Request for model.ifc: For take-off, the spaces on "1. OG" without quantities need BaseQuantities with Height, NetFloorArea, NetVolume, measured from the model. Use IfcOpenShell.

First a look at what the model holds.

```python
import ifcopenshell
import ifcopenshell.util.element
import ifcopenshell.util.unit

model = ifcopenshell.open("model.ifc")
print(model.schema)
for unit_type in ("LENGTHUNIT", "AREAUNIT", "VOLUMEUNIT"):
    print(unit_type, ifcopenshell.util.unit.calculate_unit_scale(model, unit_type))
storey = next(s for s in model.by_type("IfcBuildingStorey") if s.Name == "1. OG")
spaces = [e for e in ifcopenshell.util.element.get_decomposition(storey) if e.is_a("IfcSpace")]
for e in sorted(spaces, key=lambda e: e.id()):
    print(e.id(), e.is_a(), e.Name, list(ifcopenshell.util.element.get_psets(e, qtos_only=True)), sep=" | ")
```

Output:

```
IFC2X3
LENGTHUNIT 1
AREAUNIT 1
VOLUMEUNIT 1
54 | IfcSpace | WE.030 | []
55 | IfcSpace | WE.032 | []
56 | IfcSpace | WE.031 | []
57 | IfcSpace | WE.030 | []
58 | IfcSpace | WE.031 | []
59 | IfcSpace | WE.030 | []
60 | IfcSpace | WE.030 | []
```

```python
import ifcopenshell
import ifcopenshell.api.pset
import ifcopenshell.geom
import ifcopenshell.util.element
import ifcopenshell.util.shape
import ifcopenshell.util.unit

model = ifcopenshell.open("model.ifc")
unit_scale = ifcopenshell.util.unit.calculate_unit_scale(model)
area_scale = ifcopenshell.util.unit.calculate_unit_scale(model, "AREAUNIT")
volume_scale = ifcopenshell.util.unit.calculate_unit_scale(model, "VOLUMEUNIT")
settings = ifcopenshell.geom.settings()

storey = next(s for s in model.by_type("IfcBuildingStorey") if s.Name == "1. OG")
spaces = [e for e in ifcopenshell.util.element.get_decomposition(storey) if e.is_a("IfcSpace")]

for e in sorted(spaces, key=lambda e: e.id()):
    if ifcopenshell.util.element.get_psets(e, qtos_only=True, should_inherit=False):
        continue
    # Geometry comes back in metres, in the element's own axes.
    shape = ifcopenshell.geom.create_shape(settings, e)
    values = {
        "Height": ifcopenshell.util.shape.get_z(shape.geometry) / unit_scale,
        "NetFloorArea": ifcopenshell.util.shape.get_footprint_area(shape.geometry) / area_scale,
        "NetVolume": ifcopenshell.util.shape.get_volume(shape.geometry) / volume_scale,
    }
    qto = ifcopenshell.api.pset.add_qto(model, product=e, name="BaseQuantities")
    ifcopenshell.api.pset.edit_qto(model, qto=qto, properties=values)
    print(e.id(), {k: round(v, 3) for k, v in values.items()})

model.write("model_rev.ifc")
```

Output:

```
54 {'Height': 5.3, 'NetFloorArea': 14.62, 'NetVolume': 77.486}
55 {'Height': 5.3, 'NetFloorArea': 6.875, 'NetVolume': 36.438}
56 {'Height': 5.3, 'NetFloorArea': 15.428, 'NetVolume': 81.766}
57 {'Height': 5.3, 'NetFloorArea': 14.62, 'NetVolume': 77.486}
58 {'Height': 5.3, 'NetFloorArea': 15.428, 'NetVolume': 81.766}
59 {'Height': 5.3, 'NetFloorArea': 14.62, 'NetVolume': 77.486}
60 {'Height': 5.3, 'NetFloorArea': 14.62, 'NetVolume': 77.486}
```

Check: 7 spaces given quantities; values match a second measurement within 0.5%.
